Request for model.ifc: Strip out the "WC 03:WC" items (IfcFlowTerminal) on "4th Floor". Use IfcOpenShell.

First a look at what the model holds.

```python
import ifcopenshell
import ifcopenshell.util.element

model = ifcopenshell.open("model.ifc")
print(model.schema)
storey = next(s for s in model.by_type("IfcBuildingStorey") if s.Name == "4th Floor")
terminals = [e for e in ifcopenshell.util.element.get_decomposition(storey) if e.is_a("IfcFlowTerminal")]
seen = {}
for e in terminals:
    element_type = ifcopenshell.util.element.get_type(e)
    name = element_type.Name if element_type not in (None, e) else None
    seen[name] = seen.get(name, 0) + 1
for name, count in sorted(seen.items(), key=str):
    print(count, "x", name)
```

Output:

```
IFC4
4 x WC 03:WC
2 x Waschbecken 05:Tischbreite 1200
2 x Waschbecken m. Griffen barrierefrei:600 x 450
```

```python
import ifcopenshell
import ifcopenshell.api.root
import ifcopenshell.util.element

model = ifcopenshell.open("model.ifc")

storey = next(s for s in model.by_type("IfcBuildingStorey") if s.Name == "4th Floor")
terminals = [e for e in ifcopenshell.util.element.get_decomposition(storey) if e.is_a("IfcFlowTerminal")]
targets = [e for e in terminals if (t := ifcopenshell.util.element.get_type(e)) not in (None, e) and t.Name == "WC 03:WC"]

for e in targets:
    ifcopenshell.api.root.remove_product(model, product=e)
print(len(targets), "removed")

model.write("model_updated.ifc")
```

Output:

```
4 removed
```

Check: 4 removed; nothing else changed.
